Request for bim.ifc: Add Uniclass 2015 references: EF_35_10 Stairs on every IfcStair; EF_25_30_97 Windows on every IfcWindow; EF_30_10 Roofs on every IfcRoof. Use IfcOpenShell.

First a look at what the model holds.

```python
import ifcopenshell

model = ifcopenshell.open("bim.ifc")
print(model.schema)
print("classifications:", [c.Name for c in model.by_type("IfcClassification")])
for ifc_class in ("IfcDoor", "IfcRoof", "IfcStair", "IfcWall", "IfcWindow"):
    print(ifc_class, len(model.by_type(ifc_class)))
```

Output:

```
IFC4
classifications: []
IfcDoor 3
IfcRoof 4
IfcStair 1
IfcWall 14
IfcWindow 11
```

```python
import ifcopenshell
import ifcopenshell.api.classification

model = ifcopenshell.open("bim.ifc")

system = ifcopenshell.api.classification.add_classification(model, classification="Uniclass 2015")

codes = {
    "IfcStair": ("EF_35_10", "Stairs"),
    "IfcWindow": ("EF_25_30_97", "Windows"),
    "IfcRoof": ("EF_30_10", "Roofs"),
}
for ifc_class, (code, name) in codes.items():
    products = model.by_type(ifc_class)
    ifcopenshell.api.classification.add_reference(
        model, products=products, classification=system, identification=code, name=name
    )
    print(code, len(products))

model.write("bim-out.ifc")
```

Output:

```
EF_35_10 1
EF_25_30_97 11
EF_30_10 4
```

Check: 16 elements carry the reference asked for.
